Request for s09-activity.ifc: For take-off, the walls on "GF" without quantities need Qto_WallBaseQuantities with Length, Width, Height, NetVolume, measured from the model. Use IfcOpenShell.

First a look at what the model holds.

```python
import ifcopenshell
import ifcopenshell.util.element
import ifcopenshell.util.unit

model = ifcopenshell.open("s09-activity.ifc")
print(model.schema)
for unit_type in ("LENGTHUNIT", "AREAUNIT", "VOLUMEUNIT"):
    print(unit_type, ifcopenshell.util.unit.calculate_unit_scale(model, unit_type))
storey = next(s for s in model.by_type("IfcBuildingStorey") if s.Name == "GF")
walls = [e for e in ifcopenshell.util.element.get_decomposition(storey) if e.is_a("IfcWall")]
for e in sorted(walls, key=lambda e: e.id()):
    print(e.id(), e.is_a(), e.Name, list(ifcopenshell.util.element.get_psets(e, qtos_only=True)), sep=" | ")
```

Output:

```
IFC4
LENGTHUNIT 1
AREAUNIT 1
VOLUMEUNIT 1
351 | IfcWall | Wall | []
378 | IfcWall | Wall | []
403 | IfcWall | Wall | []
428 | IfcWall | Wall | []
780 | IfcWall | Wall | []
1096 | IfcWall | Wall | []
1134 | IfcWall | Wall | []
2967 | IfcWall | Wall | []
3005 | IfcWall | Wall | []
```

```python
import ifcopenshell
import ifcopenshell.api.pset
import ifcopenshell.geom
import ifcopenshell.util.element
import ifcopenshell.util.shape
import ifcopenshell.util.unit

model = ifcopenshell.open("s09-activity.ifc")
unit_scale = ifcopenshell.util.unit.calculate_unit_scale(model)
volume_scale = ifcopenshell.util.unit.calculate_unit_scale(model, "VOLUMEUNIT")
settings = ifcopenshell.geom.settings()

storey = next(s for s in model.by_type("IfcBuildingStorey") if s.Name == "GF")
walls = [e for e in ifcopenshell.util.element.get_decomposition(storey) if e.is_a("IfcWall")]

for e in sorted(walls, key=lambda e: e.id()):
    if ifcopenshell.util.element.get_psets(e, qtos_only=True, should_inherit=False):
        continue
    # Geometry comes back in metres, in the element's own axes.
    shape = ifcopenshell.geom.create_shape(settings, e)
    values = {
        "Length": ifcopenshell.util.shape.get_x(shape.geometry) / unit_scale,
        "Width": ifcopenshell.util.shape.get_y(shape.geometry) / unit_scale,
        "Height": ifcopenshell.util.shape.get_z(shape.geometry) / unit_scale,
        "NetVolume": ifcopenshell.util.shape.get_volume(shape.geometry) / volume_scale,
    }
    qto = ifcopenshell.api.pset.add_qto(model, product=e, name="Qto_WallBaseQuantities")
    ifcopenshell.api.pset.edit_qto(model, qto=qto, properties=values)
    print(e.id(), {k: round(v, 3) for k, v in values.items()})

model.write("s09-activity_v2.ifc")
```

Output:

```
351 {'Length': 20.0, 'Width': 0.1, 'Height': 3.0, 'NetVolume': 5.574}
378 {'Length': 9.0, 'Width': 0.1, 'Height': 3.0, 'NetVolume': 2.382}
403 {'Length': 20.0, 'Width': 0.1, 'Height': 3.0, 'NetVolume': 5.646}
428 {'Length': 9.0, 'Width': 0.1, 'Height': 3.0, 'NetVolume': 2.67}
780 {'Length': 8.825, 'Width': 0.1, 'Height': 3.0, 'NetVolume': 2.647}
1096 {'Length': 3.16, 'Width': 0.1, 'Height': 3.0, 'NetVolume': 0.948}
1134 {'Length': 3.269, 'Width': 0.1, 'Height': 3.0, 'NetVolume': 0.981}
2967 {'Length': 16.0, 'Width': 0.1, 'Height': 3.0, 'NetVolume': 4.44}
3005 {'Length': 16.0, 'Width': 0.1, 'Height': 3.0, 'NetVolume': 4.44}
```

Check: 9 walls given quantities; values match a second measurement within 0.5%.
